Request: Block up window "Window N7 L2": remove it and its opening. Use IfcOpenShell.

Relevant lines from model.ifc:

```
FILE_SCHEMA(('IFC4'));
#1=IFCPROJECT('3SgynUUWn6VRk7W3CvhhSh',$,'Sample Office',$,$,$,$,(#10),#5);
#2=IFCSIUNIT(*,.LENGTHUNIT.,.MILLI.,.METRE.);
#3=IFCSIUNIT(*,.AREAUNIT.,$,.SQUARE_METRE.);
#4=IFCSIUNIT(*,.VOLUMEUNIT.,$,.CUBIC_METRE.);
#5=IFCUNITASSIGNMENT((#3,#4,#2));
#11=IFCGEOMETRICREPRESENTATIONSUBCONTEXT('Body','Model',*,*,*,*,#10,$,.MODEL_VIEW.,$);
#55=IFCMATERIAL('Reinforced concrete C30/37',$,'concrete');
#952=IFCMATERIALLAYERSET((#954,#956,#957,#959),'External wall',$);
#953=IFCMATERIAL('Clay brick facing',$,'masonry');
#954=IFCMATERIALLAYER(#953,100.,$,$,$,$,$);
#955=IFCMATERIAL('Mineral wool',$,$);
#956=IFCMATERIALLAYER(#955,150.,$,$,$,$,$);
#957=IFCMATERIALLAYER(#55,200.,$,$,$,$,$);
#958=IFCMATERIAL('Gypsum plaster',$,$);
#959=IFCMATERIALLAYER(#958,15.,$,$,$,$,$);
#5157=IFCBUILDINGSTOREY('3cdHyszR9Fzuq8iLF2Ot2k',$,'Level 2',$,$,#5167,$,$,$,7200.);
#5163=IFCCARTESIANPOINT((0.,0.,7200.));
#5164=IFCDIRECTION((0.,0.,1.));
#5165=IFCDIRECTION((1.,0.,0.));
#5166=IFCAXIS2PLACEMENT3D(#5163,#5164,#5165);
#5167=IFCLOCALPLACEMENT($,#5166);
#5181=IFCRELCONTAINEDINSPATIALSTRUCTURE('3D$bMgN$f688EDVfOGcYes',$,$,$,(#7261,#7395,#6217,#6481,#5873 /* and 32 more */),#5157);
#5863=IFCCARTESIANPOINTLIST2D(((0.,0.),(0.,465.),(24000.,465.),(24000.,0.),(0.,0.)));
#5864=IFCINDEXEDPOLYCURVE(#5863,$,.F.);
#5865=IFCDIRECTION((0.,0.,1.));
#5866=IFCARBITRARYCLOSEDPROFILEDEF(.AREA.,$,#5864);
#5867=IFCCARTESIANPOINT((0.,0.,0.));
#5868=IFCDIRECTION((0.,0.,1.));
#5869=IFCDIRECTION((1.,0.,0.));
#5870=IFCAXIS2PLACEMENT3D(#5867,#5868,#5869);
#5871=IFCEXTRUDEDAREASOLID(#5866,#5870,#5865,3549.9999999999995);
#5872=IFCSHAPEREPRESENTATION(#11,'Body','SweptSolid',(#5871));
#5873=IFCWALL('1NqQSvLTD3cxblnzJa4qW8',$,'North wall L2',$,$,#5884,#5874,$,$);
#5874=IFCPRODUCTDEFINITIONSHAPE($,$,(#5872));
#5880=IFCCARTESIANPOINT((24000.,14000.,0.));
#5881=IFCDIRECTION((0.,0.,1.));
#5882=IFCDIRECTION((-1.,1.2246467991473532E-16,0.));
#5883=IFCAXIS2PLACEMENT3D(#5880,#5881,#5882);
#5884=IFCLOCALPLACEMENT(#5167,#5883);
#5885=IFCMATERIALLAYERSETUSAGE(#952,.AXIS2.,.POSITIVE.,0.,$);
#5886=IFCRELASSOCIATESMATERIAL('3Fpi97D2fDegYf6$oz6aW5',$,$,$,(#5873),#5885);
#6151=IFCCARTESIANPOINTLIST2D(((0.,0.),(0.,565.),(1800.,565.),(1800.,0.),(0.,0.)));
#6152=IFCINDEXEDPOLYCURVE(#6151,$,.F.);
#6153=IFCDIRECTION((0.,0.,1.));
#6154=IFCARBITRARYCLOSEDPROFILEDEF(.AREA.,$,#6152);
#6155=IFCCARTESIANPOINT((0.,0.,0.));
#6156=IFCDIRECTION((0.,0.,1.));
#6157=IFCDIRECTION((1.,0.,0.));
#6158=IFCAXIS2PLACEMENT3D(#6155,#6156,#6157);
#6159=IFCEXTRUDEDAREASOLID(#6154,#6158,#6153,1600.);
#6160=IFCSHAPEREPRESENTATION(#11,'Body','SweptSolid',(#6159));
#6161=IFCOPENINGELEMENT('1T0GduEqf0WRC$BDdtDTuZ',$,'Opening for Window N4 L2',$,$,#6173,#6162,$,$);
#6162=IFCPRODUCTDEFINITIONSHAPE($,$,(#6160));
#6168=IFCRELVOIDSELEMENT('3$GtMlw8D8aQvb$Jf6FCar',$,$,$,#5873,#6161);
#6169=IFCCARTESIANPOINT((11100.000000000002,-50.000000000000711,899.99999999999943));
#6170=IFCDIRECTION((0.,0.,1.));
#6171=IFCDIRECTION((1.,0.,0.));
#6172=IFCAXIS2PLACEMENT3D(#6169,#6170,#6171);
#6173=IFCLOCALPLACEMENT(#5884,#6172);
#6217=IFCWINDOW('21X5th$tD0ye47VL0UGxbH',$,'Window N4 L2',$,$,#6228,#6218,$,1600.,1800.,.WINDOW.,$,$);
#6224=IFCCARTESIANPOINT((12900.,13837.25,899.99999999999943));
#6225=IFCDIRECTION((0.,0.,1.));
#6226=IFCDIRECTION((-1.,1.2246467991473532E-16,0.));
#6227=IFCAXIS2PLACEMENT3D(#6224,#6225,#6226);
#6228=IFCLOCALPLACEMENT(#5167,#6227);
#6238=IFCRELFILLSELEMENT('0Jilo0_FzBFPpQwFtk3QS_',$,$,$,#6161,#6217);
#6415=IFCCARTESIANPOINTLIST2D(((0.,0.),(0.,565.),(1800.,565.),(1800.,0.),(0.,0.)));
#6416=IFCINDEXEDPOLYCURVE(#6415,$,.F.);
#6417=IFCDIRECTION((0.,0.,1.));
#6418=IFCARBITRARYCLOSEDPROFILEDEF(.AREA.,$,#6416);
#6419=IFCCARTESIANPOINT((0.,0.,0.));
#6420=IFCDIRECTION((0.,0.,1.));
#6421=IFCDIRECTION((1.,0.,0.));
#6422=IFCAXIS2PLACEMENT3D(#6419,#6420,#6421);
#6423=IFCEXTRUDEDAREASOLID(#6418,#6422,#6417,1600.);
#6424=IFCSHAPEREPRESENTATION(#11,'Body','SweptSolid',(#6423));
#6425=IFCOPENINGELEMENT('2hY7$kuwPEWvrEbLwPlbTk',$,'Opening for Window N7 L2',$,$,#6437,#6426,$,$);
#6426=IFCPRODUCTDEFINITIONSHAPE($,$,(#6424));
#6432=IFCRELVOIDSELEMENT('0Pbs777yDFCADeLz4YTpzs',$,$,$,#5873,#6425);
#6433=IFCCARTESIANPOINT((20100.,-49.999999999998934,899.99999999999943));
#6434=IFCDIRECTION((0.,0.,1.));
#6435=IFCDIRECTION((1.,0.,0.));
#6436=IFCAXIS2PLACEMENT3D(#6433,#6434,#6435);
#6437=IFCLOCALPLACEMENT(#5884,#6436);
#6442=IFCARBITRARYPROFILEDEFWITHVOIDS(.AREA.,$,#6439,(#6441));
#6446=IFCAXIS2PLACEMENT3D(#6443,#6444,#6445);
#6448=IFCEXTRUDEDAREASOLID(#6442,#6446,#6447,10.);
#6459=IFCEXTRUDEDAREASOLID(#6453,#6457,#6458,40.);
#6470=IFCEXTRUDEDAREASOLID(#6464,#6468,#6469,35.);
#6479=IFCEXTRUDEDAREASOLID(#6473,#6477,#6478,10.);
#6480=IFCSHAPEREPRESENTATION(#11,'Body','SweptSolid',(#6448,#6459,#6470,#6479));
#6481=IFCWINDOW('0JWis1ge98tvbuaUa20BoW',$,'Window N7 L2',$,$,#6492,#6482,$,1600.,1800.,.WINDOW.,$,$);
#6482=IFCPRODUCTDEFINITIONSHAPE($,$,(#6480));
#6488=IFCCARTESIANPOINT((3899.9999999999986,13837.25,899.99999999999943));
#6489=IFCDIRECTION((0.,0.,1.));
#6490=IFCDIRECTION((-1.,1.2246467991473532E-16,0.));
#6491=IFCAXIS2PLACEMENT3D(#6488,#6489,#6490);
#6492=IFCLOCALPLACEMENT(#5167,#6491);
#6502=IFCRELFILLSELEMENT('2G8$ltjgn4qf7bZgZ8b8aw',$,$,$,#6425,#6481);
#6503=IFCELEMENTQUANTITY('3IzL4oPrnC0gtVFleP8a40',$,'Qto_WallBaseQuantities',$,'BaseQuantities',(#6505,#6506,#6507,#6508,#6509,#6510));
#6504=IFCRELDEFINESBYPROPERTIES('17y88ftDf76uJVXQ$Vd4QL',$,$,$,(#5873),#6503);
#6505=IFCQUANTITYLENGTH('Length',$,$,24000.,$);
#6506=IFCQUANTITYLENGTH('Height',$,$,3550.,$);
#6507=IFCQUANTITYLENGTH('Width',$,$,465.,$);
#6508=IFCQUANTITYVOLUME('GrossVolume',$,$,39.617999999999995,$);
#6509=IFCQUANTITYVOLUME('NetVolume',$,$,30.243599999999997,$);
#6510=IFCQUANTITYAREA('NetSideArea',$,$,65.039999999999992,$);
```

```python
import ifcopenshell
import ifcopenshell.api.feature
import ifcopenshell.api.pset
import ifcopenshell.api.root
import ifcopenshell.geom
import ifcopenshell.util.element
import ifcopenshell.util.shape
import ifcopenshell.util.unit

model = ifcopenshell.open("model.ifc")
area_scale = ifcopenshell.util.unit.calculate_unit_scale(model, "AREAUNIT")
volume_scale = ifcopenshell.util.unit.calculate_unit_scale(model, "VOLUMEUNIT")
settings = ifcopenshell.geom.settings()


def volume(element):
    """Net volume in cubic metres, openings subtracted."""
    shape = ifcopenshell.geom.create_shape(settings, element)
    return ifcopenshell.util.shape.get_volume(shape.geometry)


window = model.by_guid("0JWis1ge98tvbuaUa20BoW")
opening = window.FillsVoids[0].RelatingOpeningElement
wall = opening.VoidsElements[0].RelatingBuildingElement
before = volume(wall)

ifcopenshell.api.root.remove_product(model, product=window)
ifcopenshell.api.feature.remove_feature(model, feature=opening)

after = volume(wall)
thickness = 0.465  # wall thickness in metres

# Update the wall's stored quantities.
qto = model.by_id(ifcopenshell.util.element.get_pset(wall, "Qto_WallBaseQuantities", should_inherit=False)["id"])
ifcopenshell.api.pset.edit_qto(model, qto=qto, properties={
    "NetVolume": after / volume_scale,
    "NetSideArea": after / thickness / area_scale,
})

print(f"wall volume {before:.3f} -> {after:.3f} m3")

model.write("model-out.ifc")
```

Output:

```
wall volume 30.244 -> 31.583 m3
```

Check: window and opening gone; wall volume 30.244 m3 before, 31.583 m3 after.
